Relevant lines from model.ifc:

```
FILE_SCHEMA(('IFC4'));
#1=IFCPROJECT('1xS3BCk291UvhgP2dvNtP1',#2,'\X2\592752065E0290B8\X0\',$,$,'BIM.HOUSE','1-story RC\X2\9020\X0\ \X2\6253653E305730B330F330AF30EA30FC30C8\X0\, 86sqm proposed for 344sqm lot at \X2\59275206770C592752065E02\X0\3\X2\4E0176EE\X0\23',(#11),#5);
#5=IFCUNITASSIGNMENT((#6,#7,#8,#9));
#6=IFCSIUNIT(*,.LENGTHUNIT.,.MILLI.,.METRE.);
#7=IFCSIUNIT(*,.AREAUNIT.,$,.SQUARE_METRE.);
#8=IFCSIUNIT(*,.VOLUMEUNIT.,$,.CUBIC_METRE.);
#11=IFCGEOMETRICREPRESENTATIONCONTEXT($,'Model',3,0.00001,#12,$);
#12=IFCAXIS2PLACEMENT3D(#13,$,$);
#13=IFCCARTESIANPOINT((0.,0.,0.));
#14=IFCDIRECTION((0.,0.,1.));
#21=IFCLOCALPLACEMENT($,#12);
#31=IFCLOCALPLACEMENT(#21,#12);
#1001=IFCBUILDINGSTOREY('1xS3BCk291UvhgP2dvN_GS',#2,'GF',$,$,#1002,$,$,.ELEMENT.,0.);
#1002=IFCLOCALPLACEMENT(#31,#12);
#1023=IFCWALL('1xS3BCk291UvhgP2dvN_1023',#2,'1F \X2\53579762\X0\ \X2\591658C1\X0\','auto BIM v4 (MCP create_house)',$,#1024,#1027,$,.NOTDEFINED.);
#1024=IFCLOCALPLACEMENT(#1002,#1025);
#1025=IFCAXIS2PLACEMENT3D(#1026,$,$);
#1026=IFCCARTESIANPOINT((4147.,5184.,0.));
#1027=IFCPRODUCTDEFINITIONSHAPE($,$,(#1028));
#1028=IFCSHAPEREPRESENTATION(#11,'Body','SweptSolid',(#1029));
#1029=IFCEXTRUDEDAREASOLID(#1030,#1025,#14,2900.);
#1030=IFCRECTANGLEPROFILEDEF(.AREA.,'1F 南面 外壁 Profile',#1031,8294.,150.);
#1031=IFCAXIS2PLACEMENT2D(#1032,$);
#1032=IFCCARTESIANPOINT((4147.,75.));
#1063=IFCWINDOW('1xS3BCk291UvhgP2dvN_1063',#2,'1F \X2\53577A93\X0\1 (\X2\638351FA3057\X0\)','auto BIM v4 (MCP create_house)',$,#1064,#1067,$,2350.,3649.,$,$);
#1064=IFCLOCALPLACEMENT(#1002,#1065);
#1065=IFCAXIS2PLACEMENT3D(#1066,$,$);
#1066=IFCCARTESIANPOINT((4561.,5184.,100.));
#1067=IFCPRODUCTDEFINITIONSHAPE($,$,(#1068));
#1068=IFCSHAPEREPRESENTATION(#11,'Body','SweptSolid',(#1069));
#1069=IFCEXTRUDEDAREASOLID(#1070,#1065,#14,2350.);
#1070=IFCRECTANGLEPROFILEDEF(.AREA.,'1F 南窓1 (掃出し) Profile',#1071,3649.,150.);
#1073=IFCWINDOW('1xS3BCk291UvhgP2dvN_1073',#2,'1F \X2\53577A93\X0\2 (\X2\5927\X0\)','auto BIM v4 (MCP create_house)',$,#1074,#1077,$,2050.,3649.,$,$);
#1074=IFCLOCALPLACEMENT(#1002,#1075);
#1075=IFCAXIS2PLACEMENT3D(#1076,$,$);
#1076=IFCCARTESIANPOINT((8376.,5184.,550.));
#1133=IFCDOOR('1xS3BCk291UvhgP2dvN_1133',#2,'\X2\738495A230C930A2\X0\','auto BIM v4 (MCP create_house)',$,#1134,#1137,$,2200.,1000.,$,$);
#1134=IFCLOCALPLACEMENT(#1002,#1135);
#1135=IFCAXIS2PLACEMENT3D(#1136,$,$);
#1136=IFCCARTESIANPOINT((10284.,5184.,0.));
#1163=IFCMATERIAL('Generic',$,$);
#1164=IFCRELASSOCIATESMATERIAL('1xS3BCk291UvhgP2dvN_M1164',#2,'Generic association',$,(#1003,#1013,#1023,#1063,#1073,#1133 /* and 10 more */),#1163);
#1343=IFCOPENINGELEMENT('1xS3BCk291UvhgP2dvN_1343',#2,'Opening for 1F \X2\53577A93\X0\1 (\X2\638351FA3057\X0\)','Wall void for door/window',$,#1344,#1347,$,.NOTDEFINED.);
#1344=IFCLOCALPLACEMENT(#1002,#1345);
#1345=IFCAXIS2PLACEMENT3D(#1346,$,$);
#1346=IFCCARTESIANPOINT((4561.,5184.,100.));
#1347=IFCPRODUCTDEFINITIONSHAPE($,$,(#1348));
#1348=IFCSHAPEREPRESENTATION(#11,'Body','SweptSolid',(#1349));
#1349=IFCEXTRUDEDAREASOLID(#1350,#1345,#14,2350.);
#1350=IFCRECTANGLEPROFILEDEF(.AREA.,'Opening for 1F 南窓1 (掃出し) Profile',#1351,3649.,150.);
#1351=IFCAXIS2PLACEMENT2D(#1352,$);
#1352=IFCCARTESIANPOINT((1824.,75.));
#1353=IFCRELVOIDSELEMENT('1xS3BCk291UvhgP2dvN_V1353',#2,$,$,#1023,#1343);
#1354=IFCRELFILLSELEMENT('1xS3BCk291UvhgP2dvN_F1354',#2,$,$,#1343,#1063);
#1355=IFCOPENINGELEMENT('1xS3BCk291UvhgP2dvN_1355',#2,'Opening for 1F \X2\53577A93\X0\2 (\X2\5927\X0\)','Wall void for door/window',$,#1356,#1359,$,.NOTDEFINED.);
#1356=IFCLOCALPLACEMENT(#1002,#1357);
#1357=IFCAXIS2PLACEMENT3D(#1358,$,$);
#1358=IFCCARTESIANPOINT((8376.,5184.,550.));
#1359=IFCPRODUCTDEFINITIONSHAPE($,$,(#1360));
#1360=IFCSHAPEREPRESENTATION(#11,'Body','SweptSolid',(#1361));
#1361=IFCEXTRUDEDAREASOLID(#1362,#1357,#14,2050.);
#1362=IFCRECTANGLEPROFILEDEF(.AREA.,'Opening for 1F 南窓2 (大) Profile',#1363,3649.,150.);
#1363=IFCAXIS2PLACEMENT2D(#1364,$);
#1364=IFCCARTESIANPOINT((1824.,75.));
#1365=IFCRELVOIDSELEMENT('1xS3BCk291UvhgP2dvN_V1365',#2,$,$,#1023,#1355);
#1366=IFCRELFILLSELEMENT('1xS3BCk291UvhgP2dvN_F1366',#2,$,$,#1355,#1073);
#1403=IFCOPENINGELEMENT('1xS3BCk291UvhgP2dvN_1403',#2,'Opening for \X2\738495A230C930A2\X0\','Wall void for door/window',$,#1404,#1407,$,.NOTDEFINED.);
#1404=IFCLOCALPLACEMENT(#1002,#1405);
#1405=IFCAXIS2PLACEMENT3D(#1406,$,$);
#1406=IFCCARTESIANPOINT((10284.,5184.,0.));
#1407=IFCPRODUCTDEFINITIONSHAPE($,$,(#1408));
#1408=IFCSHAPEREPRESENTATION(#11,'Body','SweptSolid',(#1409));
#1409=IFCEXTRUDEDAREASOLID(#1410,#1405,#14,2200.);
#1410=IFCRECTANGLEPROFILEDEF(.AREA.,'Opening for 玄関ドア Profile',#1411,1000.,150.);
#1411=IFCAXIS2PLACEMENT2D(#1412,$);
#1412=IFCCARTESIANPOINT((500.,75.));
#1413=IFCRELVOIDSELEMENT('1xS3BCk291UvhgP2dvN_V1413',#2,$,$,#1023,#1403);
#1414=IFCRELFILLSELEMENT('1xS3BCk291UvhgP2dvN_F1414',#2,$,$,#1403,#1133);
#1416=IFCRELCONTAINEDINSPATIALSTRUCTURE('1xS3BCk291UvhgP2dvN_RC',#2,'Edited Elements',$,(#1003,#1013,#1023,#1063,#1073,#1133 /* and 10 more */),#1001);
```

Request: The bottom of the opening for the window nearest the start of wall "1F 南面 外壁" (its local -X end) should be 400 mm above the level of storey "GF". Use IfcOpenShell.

```python
import numpy as np
import ifcopenshell
import ifcopenshell.api.geometry
import ifcopenshell.geom
import ifcopenshell.util.element
import ifcopenshell.util.placement
import ifcopenshell.util.shape
import ifcopenshell.util.unit

model = ifcopenshell.open("model.ifc")
unit_scale = ifcopenshell.util.unit.calculate_unit_scale(model)

window = model.by_guid("1xS3BCk291UvhgP2dvN_1063")
opening = window.FillsVoids[0].RelatingOpeningElement
storey = ifcopenshell.util.element.get_container(window, ifc_class="IfcBuildingStorey")
level = ifcopenshell.util.placement.get_local_placement(storey.ObjectPlacement)[2, 3]

# The opening's origin need not be at the sill, so measure its lowest point.
shape = ifcopenshell.geom.create_shape(ifcopenshell.geom.settings(), opening)
bottom = ifcopenshell.util.shape.get_shape_bottom_elevation(shape, shape.geometry) / unit_scale
dz = level + 400.0 - bottom

shift = np.array([0.0, 0.0, dz])
# The window is not placed relative to its opening, so move both.
for product in (opening, window):
    matrix = ifcopenshell.util.placement.get_local_placement(product.ObjectPlacement)
    matrix[:3, 3] += shift
    ifcopenshell.api.geometry.edit_object_placement(model, product=product, matrix=matrix, is_si=False)

print(f"moved by {dz * unit_scale:+.3f} m")

model.write("model_edited.ifc")
```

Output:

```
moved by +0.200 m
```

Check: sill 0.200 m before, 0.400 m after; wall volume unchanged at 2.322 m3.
